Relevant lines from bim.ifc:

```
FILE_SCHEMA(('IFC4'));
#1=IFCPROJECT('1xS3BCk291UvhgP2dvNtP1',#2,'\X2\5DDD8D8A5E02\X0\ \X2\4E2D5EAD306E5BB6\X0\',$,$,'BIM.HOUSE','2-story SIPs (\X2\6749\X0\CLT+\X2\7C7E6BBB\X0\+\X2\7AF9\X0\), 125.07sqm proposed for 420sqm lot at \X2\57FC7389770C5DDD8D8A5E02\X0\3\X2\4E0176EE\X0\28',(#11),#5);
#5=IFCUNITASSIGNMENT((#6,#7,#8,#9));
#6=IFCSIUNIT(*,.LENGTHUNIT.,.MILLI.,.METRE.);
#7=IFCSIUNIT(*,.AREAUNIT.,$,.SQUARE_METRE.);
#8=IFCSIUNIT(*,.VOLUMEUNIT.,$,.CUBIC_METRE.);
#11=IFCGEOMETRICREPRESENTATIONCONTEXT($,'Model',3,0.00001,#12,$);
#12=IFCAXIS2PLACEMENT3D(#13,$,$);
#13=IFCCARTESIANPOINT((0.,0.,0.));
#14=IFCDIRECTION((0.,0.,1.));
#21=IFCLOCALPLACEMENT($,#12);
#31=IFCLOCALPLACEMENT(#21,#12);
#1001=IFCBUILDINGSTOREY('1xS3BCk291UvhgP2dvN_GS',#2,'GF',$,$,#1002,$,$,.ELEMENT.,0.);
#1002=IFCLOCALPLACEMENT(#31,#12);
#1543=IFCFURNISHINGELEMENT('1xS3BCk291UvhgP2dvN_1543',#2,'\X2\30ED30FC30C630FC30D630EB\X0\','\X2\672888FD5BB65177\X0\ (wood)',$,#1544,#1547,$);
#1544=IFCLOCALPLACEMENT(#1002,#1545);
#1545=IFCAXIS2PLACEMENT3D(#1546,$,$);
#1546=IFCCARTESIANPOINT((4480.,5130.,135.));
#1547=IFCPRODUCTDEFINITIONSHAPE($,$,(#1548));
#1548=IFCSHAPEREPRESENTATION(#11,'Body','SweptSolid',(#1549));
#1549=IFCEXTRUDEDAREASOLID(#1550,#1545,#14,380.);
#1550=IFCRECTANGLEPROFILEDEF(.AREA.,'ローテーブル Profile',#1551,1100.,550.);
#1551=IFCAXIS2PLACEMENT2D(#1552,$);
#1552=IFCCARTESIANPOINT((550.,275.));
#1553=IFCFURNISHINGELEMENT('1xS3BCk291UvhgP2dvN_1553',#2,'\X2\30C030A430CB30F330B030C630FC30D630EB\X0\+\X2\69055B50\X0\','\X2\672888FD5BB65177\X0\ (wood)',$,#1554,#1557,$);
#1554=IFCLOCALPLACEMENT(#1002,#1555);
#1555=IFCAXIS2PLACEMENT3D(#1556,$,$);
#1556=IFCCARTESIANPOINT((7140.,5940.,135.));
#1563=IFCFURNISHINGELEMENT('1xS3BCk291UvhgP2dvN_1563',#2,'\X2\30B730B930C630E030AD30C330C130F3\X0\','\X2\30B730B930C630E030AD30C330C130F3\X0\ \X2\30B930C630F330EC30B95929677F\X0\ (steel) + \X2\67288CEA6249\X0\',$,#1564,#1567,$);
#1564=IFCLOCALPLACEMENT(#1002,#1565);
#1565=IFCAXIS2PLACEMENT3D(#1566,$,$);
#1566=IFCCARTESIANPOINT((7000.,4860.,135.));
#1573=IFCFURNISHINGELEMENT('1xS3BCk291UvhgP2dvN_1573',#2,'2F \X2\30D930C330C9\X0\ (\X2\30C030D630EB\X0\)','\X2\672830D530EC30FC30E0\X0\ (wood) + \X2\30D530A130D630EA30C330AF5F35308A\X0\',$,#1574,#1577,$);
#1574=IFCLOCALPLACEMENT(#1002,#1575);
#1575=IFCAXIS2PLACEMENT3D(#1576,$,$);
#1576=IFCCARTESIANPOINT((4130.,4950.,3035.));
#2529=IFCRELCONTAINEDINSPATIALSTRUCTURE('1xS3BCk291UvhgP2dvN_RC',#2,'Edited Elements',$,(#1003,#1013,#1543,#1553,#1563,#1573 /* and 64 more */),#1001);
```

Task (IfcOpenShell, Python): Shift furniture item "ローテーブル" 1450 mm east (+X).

```python
import ifcopenshell
import ifcopenshell.api.geometry
import ifcopenshell.util.placement

model = ifcopenshell.open("bim.ifc")

item = model.by_guid("1xS3BCk291UvhgP2dvN_1543")
matrix = ifcopenshell.util.placement.get_local_placement(item.ObjectPlacement)
matrix[0, 3] += 1450.0
ifcopenshell.api.geometry.edit_object_placement(model, product=item, matrix=matrix, is_si=False)

print(ifcopenshell.util.placement.get_local_placement(item.ObjectPlacement).round(3) + 0.0)

model.write("bim_rev.ifc")
```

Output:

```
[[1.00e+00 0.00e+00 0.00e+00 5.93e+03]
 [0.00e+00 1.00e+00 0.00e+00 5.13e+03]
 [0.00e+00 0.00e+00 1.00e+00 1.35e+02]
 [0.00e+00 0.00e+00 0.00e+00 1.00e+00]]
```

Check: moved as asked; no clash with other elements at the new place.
